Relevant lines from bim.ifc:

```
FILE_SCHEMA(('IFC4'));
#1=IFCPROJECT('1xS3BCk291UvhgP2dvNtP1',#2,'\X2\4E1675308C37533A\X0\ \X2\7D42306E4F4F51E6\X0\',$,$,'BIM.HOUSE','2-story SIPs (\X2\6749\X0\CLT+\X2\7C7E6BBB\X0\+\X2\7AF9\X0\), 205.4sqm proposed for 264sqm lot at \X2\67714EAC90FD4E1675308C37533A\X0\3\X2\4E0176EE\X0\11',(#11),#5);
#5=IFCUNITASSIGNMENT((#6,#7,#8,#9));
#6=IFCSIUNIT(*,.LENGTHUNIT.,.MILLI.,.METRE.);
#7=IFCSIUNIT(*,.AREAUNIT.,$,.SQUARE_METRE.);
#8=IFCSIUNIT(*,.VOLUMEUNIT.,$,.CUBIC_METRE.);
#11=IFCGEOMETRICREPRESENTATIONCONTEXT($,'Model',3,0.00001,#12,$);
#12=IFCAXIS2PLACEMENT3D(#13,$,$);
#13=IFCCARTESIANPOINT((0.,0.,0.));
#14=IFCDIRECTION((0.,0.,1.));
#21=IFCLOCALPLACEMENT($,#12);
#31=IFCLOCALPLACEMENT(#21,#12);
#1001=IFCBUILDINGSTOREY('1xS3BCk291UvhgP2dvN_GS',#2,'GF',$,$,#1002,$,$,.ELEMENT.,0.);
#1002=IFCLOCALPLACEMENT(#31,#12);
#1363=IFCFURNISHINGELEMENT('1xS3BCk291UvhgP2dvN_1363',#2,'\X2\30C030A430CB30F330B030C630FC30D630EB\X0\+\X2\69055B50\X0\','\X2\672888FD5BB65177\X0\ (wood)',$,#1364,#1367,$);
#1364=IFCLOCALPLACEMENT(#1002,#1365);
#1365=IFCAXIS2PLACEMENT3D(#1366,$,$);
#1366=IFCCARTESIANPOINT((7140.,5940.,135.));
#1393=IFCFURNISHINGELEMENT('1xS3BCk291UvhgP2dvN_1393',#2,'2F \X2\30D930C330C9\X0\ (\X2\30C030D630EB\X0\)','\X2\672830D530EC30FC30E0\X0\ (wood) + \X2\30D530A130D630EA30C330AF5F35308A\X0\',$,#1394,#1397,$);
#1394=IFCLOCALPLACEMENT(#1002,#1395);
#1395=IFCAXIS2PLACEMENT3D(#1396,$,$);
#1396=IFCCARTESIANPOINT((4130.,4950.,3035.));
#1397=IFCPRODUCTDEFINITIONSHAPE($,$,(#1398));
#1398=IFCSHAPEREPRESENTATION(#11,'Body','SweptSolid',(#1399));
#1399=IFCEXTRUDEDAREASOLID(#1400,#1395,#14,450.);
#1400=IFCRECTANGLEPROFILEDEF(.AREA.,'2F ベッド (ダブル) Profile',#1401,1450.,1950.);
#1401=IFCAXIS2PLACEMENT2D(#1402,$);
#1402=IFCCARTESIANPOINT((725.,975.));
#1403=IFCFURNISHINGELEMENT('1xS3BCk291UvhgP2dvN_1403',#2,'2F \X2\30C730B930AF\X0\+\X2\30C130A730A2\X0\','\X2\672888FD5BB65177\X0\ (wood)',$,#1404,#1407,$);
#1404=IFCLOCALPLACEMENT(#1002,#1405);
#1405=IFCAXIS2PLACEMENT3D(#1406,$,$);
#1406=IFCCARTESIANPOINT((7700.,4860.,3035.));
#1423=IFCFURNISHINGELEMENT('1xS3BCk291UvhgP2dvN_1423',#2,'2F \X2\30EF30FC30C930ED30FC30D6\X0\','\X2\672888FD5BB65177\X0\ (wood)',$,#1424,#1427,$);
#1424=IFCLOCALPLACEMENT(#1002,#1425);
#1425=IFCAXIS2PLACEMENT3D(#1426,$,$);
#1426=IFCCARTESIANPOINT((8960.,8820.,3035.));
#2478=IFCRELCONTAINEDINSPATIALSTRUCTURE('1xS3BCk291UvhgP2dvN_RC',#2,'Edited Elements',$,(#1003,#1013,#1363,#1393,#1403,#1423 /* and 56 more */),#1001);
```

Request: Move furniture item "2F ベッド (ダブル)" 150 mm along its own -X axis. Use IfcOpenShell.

```python
import ifcopenshell
import ifcopenshell.api.geometry
import ifcopenshell.util.placement
import ifcopenshell.util.unit

model = ifcopenshell.open("bim.ifc")
unit_scale = ifcopenshell.util.unit.calculate_unit_scale(model)

item = model.by_guid("1xS3BCk291UvhgP2dvN_1393")
matrix = ifcopenshell.util.placement.get_local_placement(item.ObjectPlacement)
matrix[:3, 3] -= matrix[:3, 0] * 0.15 / unit_scale
ifcopenshell.api.geometry.edit_object_placement(model, product=item, matrix=matrix, is_si=False)

print(ifcopenshell.util.placement.get_local_placement(item.ObjectPlacement).round(3) + 0.0)

model.write("bim_edited.ifc")
```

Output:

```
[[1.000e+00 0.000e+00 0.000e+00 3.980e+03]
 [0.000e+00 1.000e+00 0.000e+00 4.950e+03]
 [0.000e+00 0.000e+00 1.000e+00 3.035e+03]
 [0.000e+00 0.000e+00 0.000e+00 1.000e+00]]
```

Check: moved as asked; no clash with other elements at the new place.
